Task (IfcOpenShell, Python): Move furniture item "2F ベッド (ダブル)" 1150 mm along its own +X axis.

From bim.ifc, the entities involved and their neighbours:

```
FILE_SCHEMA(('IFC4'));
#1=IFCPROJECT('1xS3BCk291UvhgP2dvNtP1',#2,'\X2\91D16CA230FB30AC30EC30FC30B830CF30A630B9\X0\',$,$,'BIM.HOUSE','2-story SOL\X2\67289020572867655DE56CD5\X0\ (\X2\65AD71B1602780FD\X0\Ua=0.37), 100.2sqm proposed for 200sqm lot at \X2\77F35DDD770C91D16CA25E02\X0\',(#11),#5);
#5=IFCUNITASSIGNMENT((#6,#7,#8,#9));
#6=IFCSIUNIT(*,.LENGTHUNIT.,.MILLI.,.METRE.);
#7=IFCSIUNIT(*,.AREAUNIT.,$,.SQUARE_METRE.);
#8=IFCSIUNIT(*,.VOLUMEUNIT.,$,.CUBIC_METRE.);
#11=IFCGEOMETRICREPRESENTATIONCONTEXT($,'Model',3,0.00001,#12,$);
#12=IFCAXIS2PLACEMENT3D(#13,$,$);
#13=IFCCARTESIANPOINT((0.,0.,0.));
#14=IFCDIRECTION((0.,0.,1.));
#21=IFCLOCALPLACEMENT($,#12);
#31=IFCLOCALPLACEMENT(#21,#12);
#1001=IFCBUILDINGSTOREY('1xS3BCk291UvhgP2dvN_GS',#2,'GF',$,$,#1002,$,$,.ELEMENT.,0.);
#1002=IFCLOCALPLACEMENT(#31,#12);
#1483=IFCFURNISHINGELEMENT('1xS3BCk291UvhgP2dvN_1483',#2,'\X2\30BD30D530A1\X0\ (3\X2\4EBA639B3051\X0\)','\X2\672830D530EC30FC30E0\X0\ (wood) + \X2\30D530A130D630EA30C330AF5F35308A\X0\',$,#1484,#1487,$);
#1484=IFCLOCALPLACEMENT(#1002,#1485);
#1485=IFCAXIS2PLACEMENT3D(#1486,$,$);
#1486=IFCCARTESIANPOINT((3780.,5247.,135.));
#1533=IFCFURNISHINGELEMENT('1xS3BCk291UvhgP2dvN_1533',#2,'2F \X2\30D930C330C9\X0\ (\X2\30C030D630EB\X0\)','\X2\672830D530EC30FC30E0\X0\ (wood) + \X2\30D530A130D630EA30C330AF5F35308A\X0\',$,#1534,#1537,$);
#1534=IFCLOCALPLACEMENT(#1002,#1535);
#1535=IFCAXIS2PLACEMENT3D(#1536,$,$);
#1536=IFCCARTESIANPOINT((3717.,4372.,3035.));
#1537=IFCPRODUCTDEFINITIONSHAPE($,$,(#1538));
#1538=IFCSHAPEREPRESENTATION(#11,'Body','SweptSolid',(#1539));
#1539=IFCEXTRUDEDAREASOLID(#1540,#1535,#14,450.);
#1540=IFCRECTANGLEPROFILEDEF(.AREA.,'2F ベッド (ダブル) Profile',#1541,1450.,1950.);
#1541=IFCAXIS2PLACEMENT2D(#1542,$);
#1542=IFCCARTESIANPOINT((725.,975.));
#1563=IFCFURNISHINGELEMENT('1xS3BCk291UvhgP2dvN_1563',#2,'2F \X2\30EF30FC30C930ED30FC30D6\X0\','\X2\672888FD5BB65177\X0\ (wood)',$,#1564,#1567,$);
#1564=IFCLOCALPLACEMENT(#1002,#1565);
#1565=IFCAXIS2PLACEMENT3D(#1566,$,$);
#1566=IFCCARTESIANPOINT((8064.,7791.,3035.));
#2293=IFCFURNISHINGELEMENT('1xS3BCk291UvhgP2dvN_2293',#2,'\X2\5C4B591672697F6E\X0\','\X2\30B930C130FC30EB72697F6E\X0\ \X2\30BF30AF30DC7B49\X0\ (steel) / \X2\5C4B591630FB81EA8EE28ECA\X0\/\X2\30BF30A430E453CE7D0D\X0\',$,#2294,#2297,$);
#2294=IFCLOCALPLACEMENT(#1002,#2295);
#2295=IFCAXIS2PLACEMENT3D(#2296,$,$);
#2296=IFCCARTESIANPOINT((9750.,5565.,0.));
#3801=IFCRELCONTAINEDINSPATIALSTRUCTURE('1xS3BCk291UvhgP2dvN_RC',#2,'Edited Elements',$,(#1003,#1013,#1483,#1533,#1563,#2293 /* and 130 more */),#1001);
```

```python
import ifcopenshell
import ifcopenshell.api.geometry
import ifcopenshell.util.placement
import ifcopenshell.util.unit

model = ifcopenshell.open("bim.ifc")
unit_scale = ifcopenshell.util.unit.calculate_unit_scale(model)

item = model.by_id(1533)
matrix = ifcopenshell.util.placement.get_local_placement(item.ObjectPlacement)
matrix[:3, 3] += matrix[:3, 0] * 1.15 / unit_scale
ifcopenshell.api.geometry.edit_object_placement(model, product=item, matrix=matrix, is_si=False)

print(ifcopenshell.util.placement.get_local_placement(item.ObjectPlacement).round(3) + 0.0)

model.write("bim-out.ifc")
```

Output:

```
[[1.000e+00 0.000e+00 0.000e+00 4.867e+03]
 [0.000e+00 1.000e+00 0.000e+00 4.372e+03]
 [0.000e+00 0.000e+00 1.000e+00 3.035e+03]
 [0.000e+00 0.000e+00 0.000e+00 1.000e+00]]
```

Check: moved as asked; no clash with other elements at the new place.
